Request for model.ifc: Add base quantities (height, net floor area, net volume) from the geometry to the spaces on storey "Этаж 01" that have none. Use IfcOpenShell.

First a look at what the model holds.

```python
import ifcopenshell
import ifcopenshell.util.element
import ifcopenshell.util.unit

model = ifcopenshell.open("model.ifc")
print(model.schema)
for unit_type in ("LENGTHUNIT", "AREAUNIT", "VOLUMEUNIT"):
    print(unit_type, ifcopenshell.util.unit.calculate_unit_scale(model, unit_type))
storey = next(s for s in model.by_type("IfcBuildingStorey") if s.Name == "Этаж 01")
spaces = [e for e in ifcopenshell.util.element.get_decomposition(storey) if e.is_a("IfcSpace")]
for e in sorted(spaces, key=lambda e: e.id()):
    print(e.id(), e.is_a(), e.Name, list(ifcopenshell.util.element.get_psets(e, qtos_only=True)), sep=" | ")
```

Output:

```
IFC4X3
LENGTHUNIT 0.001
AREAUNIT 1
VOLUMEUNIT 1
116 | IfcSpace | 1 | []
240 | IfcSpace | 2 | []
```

```python
import ifcopenshell
import ifcopenshell.api.pset
import ifcopenshell.geom
import ifcopenshell.util.element
import ifcopenshell.util.shape
import ifcopenshell.util.unit

model = ifcopenshell.open("model.ifc")
unit_scale = ifcopenshell.util.unit.calculate_unit_scale(model)
area_scale = ifcopenshell.util.unit.calculate_unit_scale(model, "AREAUNIT")
volume_scale = ifcopenshell.util.unit.calculate_unit_scale(model, "VOLUMEUNIT")
settings = ifcopenshell.geom.settings()

storey = next(s for s in model.by_type("IfcBuildingStorey") if s.Name == "Этаж 01")
spaces = [e for e in ifcopenshell.util.element.get_decomposition(storey) if e.is_a("IfcSpace")]

for e in sorted(spaces, key=lambda e: e.id()):
    if ifcopenshell.util.element.get_psets(e, qtos_only=True, should_inherit=False):
        continue
    # Geometry comes back in metres, in the element's own axes.
    shape = ifcopenshell.geom.create_shape(settings, e)
    values = {
        "Height": ifcopenshell.util.shape.get_z(shape.geometry) / unit_scale,
        "NetFloorArea": ifcopenshell.util.shape.get_footprint_area(shape.geometry) / area_scale,
        "NetVolume": ifcopenshell.util.shape.get_volume(shape.geometry) / volume_scale,
    }
    qto = ifcopenshell.api.pset.add_qto(model, product=e, name="Qto_SpaceBaseQuantities")
    ifcopenshell.api.pset.edit_qto(model, qto=qto, properties=values)
    print(e.id(), {k: round(v, 3) for k, v in values.items()})

model.write("model_v2.ifc")
```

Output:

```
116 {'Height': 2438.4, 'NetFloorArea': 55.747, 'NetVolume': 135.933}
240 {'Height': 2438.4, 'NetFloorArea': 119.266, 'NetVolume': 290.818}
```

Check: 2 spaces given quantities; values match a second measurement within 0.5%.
